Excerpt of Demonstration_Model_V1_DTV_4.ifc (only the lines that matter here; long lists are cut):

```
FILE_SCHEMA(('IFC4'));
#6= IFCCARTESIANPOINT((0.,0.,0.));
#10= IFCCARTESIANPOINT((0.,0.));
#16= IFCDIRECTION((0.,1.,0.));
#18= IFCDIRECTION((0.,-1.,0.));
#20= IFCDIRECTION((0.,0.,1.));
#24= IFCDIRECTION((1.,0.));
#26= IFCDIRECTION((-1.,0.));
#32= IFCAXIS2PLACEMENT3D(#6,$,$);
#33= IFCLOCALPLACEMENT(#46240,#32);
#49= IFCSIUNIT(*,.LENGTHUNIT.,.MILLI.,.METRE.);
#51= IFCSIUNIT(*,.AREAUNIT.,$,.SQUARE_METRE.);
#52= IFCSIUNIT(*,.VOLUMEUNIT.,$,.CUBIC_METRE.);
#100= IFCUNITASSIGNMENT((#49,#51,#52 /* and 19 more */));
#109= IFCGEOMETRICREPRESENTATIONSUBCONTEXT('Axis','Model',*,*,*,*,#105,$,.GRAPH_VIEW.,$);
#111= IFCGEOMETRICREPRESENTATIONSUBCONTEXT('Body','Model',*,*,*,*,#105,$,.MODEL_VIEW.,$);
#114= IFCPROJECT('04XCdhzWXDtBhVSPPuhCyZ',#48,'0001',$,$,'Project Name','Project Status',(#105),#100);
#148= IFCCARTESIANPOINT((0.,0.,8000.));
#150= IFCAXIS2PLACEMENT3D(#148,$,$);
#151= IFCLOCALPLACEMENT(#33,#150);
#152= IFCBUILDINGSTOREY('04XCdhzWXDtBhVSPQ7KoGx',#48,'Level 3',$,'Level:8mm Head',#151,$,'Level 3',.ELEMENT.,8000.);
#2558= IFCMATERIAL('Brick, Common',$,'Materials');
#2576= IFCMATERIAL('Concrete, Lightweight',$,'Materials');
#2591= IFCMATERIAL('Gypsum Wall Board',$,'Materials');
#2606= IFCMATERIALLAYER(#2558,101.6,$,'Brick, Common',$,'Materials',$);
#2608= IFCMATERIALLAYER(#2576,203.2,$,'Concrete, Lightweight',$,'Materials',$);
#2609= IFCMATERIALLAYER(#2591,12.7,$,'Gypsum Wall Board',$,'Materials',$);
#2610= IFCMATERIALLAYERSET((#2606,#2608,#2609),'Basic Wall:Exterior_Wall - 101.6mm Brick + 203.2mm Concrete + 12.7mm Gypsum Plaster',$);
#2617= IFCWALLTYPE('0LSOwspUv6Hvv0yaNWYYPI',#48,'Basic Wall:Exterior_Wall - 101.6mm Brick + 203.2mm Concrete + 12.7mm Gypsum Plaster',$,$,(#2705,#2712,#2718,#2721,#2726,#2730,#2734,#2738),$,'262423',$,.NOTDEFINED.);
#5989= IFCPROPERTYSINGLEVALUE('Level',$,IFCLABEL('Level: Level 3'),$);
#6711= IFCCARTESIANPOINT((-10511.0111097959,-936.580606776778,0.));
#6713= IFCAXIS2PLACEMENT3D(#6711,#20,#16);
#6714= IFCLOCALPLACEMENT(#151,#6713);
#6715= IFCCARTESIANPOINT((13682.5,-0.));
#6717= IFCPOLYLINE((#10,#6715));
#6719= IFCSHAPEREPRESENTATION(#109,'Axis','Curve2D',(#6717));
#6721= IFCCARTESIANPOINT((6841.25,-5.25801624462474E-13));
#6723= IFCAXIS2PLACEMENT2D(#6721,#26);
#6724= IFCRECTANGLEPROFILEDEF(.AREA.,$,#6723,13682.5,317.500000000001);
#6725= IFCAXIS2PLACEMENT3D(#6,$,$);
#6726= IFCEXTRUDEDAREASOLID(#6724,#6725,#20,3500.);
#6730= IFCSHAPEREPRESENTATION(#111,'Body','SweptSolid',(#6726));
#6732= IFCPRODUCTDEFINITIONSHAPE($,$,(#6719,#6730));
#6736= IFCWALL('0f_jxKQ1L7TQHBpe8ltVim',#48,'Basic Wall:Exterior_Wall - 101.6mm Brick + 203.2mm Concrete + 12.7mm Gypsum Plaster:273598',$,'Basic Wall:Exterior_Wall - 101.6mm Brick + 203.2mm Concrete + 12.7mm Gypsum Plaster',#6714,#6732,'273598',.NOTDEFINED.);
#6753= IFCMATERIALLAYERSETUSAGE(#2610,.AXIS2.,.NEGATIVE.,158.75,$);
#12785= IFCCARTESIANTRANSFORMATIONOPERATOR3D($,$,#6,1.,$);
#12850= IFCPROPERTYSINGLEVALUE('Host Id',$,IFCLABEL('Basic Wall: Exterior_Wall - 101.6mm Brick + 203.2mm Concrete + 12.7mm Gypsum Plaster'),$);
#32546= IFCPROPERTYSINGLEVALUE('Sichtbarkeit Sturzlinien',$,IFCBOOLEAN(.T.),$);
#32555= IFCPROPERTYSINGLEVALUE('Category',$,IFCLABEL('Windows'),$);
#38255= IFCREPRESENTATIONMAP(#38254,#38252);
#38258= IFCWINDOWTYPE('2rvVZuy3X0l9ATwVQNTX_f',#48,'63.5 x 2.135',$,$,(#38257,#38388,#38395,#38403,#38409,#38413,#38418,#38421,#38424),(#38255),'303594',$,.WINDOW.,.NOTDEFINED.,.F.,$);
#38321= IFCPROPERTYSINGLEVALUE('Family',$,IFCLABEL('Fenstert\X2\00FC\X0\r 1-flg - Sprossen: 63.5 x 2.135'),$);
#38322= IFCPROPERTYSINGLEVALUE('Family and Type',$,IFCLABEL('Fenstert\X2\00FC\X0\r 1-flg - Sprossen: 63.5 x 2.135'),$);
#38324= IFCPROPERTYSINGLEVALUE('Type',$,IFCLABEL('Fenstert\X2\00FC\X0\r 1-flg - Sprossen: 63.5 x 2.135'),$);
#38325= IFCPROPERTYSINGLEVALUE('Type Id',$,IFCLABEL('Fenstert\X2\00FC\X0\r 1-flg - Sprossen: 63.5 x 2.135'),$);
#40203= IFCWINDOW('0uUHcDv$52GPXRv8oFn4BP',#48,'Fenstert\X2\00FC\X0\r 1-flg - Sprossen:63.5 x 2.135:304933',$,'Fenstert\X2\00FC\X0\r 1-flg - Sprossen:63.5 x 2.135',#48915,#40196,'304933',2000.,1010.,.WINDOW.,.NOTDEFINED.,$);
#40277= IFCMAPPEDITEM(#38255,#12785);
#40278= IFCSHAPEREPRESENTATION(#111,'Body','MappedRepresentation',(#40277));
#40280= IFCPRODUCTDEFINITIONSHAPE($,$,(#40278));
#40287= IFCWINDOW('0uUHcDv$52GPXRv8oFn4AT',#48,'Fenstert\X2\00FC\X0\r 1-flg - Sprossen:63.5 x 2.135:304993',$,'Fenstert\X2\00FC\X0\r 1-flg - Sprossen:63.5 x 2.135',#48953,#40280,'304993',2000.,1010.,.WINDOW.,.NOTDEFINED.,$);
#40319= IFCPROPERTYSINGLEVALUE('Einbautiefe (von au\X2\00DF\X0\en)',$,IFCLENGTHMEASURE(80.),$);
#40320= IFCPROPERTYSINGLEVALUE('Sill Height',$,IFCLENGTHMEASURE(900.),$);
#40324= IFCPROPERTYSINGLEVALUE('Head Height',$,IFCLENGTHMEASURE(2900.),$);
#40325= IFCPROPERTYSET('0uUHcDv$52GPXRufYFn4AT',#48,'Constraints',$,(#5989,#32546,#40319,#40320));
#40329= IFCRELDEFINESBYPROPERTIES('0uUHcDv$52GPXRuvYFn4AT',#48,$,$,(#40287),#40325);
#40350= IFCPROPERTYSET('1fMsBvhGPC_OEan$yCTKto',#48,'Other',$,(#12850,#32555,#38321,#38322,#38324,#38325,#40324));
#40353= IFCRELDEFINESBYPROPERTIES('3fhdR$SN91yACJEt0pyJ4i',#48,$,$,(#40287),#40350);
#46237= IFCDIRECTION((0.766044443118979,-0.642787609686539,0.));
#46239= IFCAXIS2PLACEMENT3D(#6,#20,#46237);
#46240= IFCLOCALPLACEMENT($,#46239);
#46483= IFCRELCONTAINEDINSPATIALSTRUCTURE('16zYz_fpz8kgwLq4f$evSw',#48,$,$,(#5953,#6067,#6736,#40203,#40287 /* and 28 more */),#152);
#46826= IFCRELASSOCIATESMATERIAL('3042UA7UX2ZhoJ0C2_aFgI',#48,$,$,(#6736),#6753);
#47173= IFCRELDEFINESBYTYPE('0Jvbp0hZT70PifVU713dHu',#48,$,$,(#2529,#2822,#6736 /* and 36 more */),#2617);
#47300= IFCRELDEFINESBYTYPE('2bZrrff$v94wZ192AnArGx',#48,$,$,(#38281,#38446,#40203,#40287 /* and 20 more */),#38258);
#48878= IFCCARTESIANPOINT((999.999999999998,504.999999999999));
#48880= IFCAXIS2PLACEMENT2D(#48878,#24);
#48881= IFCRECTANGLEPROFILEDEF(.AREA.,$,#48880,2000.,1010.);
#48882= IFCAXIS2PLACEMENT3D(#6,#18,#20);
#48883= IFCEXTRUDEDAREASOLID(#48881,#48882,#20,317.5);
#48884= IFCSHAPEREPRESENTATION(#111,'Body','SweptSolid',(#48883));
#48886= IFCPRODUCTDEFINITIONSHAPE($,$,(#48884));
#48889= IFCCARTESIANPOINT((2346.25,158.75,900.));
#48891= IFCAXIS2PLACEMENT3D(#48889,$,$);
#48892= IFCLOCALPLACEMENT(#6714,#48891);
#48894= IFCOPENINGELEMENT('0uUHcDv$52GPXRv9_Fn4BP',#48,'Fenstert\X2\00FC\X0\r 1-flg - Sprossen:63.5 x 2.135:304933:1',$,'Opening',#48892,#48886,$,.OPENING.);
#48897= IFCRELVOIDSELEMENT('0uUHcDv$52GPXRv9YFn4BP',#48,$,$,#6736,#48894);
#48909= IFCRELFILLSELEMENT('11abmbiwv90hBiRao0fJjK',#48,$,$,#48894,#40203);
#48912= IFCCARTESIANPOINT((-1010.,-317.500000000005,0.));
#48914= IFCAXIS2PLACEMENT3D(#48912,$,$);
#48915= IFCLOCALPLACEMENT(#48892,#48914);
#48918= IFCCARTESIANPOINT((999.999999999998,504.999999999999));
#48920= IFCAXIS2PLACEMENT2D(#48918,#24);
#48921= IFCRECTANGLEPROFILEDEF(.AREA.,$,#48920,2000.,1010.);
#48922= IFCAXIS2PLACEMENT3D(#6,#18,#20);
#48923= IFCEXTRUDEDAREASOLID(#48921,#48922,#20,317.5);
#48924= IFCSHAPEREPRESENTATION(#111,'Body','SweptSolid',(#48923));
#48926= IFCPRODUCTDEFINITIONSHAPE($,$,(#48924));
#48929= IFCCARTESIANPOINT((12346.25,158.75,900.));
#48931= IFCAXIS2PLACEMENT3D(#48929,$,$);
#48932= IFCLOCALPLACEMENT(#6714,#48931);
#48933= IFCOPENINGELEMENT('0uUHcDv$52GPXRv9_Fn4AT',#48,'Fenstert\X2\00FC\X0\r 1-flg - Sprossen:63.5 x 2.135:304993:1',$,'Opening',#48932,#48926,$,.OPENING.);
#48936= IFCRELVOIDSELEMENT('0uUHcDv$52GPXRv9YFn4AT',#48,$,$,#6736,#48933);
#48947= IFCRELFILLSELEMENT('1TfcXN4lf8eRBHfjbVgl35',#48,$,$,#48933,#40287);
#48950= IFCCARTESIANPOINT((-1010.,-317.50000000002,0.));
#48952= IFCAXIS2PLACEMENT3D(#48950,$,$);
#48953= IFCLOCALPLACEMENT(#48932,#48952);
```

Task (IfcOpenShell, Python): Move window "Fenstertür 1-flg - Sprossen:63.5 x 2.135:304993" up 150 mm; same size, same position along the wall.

```python
import numpy as np
import ifcopenshell
import ifcopenshell.api.geometry
import ifcopenshell.api.pset
import ifcopenshell.util.element
import ifcopenshell.util.placement
import ifcopenshell.util.unit

model = ifcopenshell.open("Demonstration_Model_V1_DTV_4.ifc")
unit_scale = ifcopenshell.util.unit.calculate_unit_scale(model)

window = model.by_id(40287)
opening = window.FillsVoids[0].RelatingOpeningElement
dz = 0.15 / unit_scale

shift = np.array([0.0, 0.0, dz])
# The window is placed relative to its opening, so it follows when the opening moves.
matrix = ifcopenshell.util.placement.get_local_placement(opening.ObjectPlacement)
matrix[:3, 3] += shift
ifcopenshell.api.geometry.edit_object_placement(
    model, product=opening, matrix=matrix, is_si=False, should_transform_children=True
)

# Keep the stored heights in step.
pset = model.by_id(ifcopenshell.util.element.get_pset(window, "Constraints", should_inherit=False)["id"])
ifcopenshell.api.pset.edit_pset(model, pset=pset, properties={
    "Sill Height": model.create_entity("IfcLengthMeasure", ifcopenshell.util.element.get_pset(window, "Constraints", "Sill Height") + dz),
})
pset = model.by_id(ifcopenshell.util.element.get_pset(window, "Other", should_inherit=False)["id"])
ifcopenshell.api.pset.edit_pset(model, pset=pset, properties={
    "Head Height": model.create_entity("IfcLengthMeasure", ifcopenshell.util.element.get_pset(window, "Other", "Head Height") + dz),
})

print(f"moved by {dz * unit_scale:+.3f} m")

model.write("Demonstration_Model_V1_DTV_4_updated.ifc")
```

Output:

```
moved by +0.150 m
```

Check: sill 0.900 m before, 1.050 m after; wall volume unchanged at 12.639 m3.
